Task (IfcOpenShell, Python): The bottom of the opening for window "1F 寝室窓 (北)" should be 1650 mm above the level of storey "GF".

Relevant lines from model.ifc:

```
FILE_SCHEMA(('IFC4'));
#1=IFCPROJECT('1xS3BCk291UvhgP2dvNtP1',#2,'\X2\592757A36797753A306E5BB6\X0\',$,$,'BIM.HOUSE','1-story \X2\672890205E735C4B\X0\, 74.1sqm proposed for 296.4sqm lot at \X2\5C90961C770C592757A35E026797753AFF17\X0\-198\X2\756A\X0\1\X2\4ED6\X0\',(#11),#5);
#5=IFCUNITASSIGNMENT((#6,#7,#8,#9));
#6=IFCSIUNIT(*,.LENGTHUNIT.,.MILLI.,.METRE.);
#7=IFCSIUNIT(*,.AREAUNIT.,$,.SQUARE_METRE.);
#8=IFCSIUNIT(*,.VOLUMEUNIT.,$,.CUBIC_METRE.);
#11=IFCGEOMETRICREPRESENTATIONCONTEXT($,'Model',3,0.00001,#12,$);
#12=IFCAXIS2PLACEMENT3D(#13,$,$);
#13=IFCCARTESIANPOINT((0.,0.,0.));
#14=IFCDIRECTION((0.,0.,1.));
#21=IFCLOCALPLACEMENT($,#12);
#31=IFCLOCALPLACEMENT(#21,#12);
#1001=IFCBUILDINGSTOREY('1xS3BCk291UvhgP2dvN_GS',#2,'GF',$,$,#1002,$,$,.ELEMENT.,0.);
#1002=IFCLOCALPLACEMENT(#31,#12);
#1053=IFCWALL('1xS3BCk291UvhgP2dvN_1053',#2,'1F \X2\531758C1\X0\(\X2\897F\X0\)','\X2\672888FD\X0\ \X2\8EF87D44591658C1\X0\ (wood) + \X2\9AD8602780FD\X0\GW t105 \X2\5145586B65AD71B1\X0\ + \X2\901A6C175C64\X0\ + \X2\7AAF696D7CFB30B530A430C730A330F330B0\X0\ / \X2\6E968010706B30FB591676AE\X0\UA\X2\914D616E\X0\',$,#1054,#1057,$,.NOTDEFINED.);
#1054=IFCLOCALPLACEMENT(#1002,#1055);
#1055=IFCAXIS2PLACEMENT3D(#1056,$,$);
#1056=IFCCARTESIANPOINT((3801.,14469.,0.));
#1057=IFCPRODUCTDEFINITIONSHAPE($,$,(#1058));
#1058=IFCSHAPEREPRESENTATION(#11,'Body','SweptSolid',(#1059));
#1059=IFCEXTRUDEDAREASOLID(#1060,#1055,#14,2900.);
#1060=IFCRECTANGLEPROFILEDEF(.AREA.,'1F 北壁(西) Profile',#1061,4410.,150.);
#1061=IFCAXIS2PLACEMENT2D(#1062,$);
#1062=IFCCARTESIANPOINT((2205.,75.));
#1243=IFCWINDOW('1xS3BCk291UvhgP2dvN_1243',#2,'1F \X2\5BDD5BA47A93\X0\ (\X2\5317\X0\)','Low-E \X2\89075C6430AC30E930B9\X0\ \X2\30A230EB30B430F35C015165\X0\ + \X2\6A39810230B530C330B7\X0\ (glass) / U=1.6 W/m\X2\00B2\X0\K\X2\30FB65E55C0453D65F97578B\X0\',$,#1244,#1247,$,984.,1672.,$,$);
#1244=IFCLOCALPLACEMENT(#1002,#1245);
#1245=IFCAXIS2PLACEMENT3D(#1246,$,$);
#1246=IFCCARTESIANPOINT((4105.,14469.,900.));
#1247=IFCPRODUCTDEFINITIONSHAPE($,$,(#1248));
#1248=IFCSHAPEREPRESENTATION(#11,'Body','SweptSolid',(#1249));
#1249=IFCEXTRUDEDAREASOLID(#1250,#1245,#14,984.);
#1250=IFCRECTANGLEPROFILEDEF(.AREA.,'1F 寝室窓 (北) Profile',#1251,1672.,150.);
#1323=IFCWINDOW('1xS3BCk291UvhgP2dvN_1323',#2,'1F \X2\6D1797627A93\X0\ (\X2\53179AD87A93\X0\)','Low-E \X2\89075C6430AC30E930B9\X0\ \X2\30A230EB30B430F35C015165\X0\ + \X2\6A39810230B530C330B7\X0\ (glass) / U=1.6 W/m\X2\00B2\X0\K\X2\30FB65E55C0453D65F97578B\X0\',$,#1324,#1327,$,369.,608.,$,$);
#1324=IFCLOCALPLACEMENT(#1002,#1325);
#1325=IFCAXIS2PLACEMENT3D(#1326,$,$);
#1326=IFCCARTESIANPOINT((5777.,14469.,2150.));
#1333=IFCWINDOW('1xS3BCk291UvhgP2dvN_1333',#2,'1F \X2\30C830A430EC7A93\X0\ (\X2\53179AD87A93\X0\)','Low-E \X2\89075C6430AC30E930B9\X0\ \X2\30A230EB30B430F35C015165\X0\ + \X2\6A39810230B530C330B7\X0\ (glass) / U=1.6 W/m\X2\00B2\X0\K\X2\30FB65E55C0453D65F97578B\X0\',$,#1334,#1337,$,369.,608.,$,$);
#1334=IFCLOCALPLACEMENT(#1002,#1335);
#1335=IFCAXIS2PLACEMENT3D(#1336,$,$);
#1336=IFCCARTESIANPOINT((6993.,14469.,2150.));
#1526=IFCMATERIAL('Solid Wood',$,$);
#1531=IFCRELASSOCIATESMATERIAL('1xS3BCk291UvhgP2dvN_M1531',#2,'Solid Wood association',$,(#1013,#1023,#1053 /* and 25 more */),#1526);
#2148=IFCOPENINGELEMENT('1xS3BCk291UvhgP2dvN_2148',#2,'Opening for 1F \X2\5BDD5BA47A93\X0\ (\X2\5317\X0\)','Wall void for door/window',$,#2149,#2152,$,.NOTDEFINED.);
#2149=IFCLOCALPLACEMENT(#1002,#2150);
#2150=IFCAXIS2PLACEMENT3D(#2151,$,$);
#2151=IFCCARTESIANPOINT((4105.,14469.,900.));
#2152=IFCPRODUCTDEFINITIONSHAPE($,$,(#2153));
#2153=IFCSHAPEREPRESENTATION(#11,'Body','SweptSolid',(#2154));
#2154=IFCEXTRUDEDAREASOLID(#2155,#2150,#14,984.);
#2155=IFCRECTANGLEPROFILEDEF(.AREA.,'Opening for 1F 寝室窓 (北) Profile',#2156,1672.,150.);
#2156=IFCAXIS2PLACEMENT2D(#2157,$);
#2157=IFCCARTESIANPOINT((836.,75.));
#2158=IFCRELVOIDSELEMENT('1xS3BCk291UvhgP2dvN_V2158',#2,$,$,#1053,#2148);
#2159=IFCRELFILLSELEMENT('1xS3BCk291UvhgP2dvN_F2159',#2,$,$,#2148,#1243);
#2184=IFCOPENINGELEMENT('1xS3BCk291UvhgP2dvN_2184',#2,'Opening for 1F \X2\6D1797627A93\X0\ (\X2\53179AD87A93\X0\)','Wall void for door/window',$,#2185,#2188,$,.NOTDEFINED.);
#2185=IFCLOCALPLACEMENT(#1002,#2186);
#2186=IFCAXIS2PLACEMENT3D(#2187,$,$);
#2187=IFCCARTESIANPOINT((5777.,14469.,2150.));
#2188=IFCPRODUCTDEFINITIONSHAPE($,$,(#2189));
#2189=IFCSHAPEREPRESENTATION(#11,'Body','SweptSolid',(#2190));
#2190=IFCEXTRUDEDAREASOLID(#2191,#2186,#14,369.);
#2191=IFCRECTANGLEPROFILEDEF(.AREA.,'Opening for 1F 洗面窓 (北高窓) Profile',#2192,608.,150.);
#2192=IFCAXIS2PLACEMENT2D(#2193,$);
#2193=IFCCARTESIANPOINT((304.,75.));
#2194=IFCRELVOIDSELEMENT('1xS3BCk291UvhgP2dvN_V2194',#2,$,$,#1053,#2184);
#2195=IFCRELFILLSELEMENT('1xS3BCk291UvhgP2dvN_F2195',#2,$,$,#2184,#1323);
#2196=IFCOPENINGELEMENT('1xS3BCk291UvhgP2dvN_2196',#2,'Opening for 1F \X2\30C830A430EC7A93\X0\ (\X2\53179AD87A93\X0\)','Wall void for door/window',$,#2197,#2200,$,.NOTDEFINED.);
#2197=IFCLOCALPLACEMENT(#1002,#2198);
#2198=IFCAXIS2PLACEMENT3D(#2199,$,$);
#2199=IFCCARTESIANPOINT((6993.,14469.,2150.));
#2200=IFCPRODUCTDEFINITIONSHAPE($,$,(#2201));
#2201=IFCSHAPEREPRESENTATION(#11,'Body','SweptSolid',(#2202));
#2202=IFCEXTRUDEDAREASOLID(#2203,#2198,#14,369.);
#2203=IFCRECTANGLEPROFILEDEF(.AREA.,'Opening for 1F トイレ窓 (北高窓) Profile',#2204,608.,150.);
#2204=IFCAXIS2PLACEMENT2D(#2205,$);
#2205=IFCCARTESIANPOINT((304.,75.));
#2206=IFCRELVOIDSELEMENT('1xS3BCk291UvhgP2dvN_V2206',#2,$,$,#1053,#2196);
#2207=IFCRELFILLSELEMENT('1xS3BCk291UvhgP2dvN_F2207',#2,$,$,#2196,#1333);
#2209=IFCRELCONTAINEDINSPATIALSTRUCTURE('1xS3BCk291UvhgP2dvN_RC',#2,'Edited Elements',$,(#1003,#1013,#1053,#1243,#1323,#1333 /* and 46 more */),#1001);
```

```python
import numpy as np
import ifcopenshell
import ifcopenshell.api.geometry
import ifcopenshell.geom
import ifcopenshell.util.element
import ifcopenshell.util.placement
import ifcopenshell.util.shape
import ifcopenshell.util.unit

model = ifcopenshell.open("model.ifc")
unit_scale = ifcopenshell.util.unit.calculate_unit_scale(model)

window = model.by_guid("1xS3BCk291UvhgP2dvN_1243")
opening = window.FillsVoids[0].RelatingOpeningElement
storey = ifcopenshell.util.element.get_container(window, ifc_class="IfcBuildingStorey")
level = ifcopenshell.util.placement.get_local_placement(storey.ObjectPlacement)[2, 3]

# The opening's origin need not be at the sill, so measure its lowest point.
shape = ifcopenshell.geom.create_shape(ifcopenshell.geom.settings(), opening)
bottom = ifcopenshell.util.shape.get_shape_bottom_elevation(shape, shape.geometry) / unit_scale
dz = level + 1.65 / unit_scale - bottom

shift = np.array([0.0, 0.0, dz])
# The window is not placed relative to its opening, so move both.
for product in (opening, window):
    matrix = ifcopenshell.util.placement.get_local_placement(product.ObjectPlacement)
    matrix[:3, 3] += shift
    ifcopenshell.api.geometry.edit_object_placement(model, product=product, matrix=matrix, is_si=False)

print(f"moved by {dz * unit_scale:+.3f} m")

model.write("model_updated.ifc")
```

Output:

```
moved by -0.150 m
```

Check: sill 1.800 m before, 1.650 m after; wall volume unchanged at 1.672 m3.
